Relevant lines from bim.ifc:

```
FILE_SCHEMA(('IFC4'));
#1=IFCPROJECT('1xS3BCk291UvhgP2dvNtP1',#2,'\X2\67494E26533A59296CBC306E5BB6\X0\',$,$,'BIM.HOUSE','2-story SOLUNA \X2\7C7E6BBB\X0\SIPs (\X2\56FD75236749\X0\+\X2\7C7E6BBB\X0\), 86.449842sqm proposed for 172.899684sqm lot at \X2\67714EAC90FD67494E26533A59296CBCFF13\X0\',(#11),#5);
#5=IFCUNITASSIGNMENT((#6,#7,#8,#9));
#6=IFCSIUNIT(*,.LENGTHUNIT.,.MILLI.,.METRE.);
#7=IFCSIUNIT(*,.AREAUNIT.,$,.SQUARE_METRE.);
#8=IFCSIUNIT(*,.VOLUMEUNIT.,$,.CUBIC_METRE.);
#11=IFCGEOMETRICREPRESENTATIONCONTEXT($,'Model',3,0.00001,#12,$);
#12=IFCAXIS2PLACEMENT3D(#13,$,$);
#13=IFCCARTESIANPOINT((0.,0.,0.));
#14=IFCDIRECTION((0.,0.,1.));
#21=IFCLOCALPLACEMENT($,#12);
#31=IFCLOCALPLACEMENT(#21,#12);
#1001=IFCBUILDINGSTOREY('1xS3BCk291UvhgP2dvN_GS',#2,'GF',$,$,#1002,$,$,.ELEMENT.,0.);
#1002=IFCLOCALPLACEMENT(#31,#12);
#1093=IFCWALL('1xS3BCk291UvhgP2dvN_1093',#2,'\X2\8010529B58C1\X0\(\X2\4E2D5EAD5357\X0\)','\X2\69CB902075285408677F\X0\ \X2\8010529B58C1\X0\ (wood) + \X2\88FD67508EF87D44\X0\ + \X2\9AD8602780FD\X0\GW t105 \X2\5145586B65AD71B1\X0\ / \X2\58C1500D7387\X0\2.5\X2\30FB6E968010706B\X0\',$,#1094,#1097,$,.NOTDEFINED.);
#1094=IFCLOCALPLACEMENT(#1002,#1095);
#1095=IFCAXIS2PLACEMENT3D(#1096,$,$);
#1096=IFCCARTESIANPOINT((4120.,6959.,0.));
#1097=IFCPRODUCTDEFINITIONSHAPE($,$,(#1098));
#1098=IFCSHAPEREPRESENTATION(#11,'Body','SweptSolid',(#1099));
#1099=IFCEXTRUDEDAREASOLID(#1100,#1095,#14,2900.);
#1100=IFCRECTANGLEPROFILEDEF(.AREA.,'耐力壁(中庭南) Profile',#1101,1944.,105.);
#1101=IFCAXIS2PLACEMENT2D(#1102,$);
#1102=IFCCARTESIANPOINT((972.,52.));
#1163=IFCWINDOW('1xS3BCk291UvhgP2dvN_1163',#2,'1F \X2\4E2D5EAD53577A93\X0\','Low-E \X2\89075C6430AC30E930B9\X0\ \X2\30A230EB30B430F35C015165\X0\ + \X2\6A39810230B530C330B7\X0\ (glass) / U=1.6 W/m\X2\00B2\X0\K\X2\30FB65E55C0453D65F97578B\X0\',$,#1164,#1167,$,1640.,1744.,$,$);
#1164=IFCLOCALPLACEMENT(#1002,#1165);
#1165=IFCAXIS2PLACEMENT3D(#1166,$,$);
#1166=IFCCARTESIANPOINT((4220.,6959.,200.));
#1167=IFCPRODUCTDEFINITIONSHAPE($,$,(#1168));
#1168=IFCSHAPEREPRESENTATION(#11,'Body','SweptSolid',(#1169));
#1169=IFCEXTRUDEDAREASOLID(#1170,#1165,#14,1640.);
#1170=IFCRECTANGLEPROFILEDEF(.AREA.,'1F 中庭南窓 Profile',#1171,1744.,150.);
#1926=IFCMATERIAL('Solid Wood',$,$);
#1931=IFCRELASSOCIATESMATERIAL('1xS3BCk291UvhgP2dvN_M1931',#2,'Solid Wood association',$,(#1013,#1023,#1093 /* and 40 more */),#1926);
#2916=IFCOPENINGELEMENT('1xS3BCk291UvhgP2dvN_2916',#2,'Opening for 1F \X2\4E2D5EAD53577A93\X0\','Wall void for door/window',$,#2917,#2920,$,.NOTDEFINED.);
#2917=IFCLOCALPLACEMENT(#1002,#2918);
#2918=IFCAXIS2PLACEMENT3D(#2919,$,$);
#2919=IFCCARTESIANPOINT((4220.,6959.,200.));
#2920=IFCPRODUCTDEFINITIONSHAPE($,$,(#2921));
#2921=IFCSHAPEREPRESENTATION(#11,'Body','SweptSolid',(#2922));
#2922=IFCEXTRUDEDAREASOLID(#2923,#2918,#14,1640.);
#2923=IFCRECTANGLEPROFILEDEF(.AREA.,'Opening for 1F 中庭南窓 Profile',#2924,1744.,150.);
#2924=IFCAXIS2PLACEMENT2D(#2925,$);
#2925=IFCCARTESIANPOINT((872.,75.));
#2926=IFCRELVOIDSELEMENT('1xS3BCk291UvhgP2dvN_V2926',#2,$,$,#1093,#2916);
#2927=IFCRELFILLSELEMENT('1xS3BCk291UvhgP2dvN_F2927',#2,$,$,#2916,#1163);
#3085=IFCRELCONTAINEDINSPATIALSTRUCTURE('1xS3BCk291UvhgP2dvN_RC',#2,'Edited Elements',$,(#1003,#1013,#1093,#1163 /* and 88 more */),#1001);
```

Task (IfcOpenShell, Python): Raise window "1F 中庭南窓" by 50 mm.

```python
import numpy as np
import ifcopenshell
import ifcopenshell.api.geometry
import ifcopenshell.util.placement
import ifcopenshell.util.unit

model = ifcopenshell.open("bim.ifc")
unit_scale = ifcopenshell.util.unit.calculate_unit_scale(model)

window = model.by_guid("1xS3BCk291UvhgP2dvN_1163")
opening = window.FillsVoids[0].RelatingOpeningElement
dz = 0.05 / unit_scale

shift = np.array([0.0, 0.0, dz])
# The window is not placed relative to its opening, so move both.
for product in (opening, window):
    matrix = ifcopenshell.util.placement.get_local_placement(product.ObjectPlacement)
    matrix[:3, 3] += shift
    ifcopenshell.api.geometry.edit_object_placement(model, product=product, matrix=matrix, is_si=False)

print(f"moved by {dz * unit_scale:+.3f} m")

model.write("bim_updated.ifc")
```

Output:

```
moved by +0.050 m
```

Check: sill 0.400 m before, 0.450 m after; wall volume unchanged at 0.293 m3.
